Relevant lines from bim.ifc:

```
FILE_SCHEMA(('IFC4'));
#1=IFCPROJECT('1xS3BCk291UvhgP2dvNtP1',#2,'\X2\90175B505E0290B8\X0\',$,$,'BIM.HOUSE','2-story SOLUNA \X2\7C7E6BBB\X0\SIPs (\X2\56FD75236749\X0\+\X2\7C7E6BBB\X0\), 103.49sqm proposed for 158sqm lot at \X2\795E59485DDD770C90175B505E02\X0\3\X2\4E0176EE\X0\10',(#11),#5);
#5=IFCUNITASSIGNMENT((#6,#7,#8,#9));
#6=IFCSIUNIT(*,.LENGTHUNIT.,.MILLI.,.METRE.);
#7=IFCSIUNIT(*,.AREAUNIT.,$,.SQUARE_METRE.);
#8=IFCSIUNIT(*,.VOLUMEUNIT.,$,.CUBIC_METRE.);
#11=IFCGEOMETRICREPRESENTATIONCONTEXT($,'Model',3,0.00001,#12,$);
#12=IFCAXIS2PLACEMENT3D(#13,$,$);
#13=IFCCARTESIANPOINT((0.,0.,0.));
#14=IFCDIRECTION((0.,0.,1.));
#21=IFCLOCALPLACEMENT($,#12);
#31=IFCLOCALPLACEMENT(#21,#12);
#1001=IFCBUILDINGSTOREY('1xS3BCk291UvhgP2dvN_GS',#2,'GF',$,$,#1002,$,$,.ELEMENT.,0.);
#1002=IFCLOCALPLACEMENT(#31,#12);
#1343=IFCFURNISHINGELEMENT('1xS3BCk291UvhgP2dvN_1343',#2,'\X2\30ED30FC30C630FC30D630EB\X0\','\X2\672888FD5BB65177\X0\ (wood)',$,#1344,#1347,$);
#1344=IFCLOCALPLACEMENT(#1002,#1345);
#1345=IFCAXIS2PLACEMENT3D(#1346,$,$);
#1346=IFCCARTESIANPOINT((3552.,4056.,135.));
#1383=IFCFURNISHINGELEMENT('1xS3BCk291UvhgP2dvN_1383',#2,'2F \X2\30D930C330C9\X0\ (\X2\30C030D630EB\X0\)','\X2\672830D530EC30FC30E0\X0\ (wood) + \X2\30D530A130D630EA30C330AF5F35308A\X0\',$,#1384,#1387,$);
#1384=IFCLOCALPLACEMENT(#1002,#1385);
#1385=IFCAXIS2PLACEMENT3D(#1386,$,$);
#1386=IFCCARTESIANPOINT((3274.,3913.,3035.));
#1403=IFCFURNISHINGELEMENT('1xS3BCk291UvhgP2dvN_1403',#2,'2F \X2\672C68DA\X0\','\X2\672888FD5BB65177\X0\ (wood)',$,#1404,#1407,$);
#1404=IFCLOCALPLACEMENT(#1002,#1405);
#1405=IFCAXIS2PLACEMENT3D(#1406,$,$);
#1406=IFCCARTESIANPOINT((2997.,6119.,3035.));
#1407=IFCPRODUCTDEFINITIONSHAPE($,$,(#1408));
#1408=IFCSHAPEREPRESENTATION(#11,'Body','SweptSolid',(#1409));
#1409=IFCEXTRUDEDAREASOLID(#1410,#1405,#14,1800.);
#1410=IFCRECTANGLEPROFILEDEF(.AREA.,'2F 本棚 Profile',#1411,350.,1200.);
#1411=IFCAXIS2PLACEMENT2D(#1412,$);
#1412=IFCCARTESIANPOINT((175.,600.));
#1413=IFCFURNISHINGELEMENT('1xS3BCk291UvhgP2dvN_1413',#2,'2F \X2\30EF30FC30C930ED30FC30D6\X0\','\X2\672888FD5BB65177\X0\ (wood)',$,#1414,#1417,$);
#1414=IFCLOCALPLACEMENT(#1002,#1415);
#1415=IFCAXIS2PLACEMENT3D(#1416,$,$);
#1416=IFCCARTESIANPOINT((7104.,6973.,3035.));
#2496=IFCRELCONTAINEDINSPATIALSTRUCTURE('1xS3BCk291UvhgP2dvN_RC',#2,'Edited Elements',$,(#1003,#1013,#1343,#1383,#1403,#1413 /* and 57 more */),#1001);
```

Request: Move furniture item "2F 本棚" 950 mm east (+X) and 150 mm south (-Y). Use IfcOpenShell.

```python
import ifcopenshell
import ifcopenshell.api.geometry
import ifcopenshell.util.placement

model = ifcopenshell.open("bim.ifc")

item = model.by_id(1403)
matrix = ifcopenshell.util.placement.get_local_placement(item.ObjectPlacement)
matrix[0, 3] += 950.0
matrix[1, 3] -= 150.0
ifcopenshell.api.geometry.edit_object_placement(model, product=item, matrix=matrix, is_si=False)

print(ifcopenshell.util.placement.get_local_placement(item.ObjectPlacement).round(3) + 0.0)

model.write("bim-out.ifc")
```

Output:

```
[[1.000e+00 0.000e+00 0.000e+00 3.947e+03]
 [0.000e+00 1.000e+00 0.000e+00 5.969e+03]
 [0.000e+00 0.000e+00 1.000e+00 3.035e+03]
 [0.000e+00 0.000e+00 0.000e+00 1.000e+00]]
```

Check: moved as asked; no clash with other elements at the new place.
